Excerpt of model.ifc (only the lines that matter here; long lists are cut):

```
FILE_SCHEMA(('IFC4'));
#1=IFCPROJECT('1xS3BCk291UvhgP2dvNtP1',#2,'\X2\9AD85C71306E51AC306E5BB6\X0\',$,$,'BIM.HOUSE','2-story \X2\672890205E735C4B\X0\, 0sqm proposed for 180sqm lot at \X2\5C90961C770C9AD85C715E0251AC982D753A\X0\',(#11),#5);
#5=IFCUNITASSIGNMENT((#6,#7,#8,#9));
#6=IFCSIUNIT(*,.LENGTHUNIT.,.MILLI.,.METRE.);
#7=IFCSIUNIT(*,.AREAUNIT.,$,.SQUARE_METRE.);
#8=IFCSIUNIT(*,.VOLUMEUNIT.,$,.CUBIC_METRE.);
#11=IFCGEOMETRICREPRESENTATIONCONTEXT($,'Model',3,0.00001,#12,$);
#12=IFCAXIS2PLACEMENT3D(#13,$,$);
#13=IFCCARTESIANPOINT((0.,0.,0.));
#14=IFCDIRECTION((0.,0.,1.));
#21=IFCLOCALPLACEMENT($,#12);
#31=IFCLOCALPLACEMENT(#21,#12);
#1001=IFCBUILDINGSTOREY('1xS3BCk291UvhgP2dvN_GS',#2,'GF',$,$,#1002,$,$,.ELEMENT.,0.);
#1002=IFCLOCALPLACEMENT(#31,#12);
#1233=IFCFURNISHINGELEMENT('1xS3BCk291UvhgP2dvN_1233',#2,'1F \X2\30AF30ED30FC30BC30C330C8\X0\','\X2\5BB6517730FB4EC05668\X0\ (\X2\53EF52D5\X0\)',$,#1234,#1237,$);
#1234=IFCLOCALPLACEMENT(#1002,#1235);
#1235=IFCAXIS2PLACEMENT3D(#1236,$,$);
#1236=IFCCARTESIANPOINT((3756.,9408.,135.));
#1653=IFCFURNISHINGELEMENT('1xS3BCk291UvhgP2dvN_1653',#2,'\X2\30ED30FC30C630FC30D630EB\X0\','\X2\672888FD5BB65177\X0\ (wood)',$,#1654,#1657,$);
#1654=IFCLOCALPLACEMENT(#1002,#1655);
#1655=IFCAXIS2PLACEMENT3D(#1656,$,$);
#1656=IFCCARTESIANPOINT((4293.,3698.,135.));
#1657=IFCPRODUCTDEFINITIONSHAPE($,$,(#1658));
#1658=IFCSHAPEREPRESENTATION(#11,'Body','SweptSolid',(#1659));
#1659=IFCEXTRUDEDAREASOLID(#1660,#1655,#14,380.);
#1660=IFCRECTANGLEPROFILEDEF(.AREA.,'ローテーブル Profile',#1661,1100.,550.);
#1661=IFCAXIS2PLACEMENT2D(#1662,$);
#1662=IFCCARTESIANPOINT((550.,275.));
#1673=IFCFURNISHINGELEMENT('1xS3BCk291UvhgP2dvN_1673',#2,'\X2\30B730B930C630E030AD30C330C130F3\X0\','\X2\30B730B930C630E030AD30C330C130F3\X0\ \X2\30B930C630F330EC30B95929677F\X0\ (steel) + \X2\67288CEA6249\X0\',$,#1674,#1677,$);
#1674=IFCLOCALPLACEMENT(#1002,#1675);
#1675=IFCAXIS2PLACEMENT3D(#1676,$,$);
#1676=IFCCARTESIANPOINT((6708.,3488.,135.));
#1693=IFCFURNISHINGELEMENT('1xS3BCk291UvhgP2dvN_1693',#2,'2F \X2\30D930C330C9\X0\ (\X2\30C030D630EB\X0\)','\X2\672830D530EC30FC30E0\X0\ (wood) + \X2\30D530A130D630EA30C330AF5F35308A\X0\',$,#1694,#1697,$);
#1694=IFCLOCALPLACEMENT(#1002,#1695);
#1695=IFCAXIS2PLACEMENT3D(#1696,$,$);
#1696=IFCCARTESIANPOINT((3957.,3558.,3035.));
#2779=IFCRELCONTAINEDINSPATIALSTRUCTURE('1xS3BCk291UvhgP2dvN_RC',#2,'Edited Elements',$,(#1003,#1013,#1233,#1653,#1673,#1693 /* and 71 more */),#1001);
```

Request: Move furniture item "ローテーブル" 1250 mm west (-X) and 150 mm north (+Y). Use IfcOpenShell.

```python
import ifcopenshell
import ifcopenshell.api.geometry
import ifcopenshell.util.placement

model = ifcopenshell.open("model.ifc")

item = model.by_guid("1xS3BCk291UvhgP2dvN_1653")
matrix = ifcopenshell.util.placement.get_local_placement(item.ObjectPlacement)
matrix[0, 3] -= 1250.0
matrix[1, 3] += 150.0
ifcopenshell.api.geometry.edit_object_placement(model, product=item, matrix=matrix, is_si=False)

print(ifcopenshell.util.placement.get_local_placement(item.ObjectPlacement).round(3) + 0.0)

model.write("model_rev.ifc")
```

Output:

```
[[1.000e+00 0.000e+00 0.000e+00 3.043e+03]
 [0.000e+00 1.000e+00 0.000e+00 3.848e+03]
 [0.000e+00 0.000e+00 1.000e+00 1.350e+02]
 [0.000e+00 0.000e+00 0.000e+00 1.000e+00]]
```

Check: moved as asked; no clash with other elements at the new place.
